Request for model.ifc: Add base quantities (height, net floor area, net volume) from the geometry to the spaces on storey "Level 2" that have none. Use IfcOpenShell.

First a look at what the model holds.

```python
import ifcopenshell
import ifcopenshell.util.element
import ifcopenshell.util.unit

model = ifcopenshell.open("model.ifc")
print(model.schema)
for unit_type in ("LENGTHUNIT", "AREAUNIT", "VOLUMEUNIT"):
    print(unit_type, ifcopenshell.util.unit.calculate_unit_scale(model, unit_type))
storey = next(s for s in model.by_type("IfcBuildingStorey") if s.Name == "Level 2")
spaces = [e for e in ifcopenshell.util.element.get_decomposition(storey) if e.is_a("IfcSpace")]
for e in sorted(spaces, key=lambda e: e.id()):
    print(e.id(), e.is_a(), e.Name, list(ifcopenshell.util.element.get_psets(e, qtos_only=True)), sep=" | ")
```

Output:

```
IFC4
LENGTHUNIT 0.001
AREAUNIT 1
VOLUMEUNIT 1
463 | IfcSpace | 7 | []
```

```python
import ifcopenshell
import ifcopenshell.api.pset
import ifcopenshell.geom
import ifcopenshell.util.element
import ifcopenshell.util.shape
import ifcopenshell.util.unit

model = ifcopenshell.open("model.ifc")
unit_scale = ifcopenshell.util.unit.calculate_unit_scale(model)
area_scale = ifcopenshell.util.unit.calculate_unit_scale(model, "AREAUNIT")
volume_scale = ifcopenshell.util.unit.calculate_unit_scale(model, "VOLUMEUNIT")
settings = ifcopenshell.geom.settings()

storey = next(s for s in model.by_type("IfcBuildingStorey") if s.Name == "Level 2")
spaces = [e for e in ifcopenshell.util.element.get_decomposition(storey) if e.is_a("IfcSpace")]

for e in sorted(spaces, key=lambda e: e.id()):
    if ifcopenshell.util.element.get_psets(e, qtos_only=True, should_inherit=False):
        continue
    # Geometry comes back in metres, in the element's own axes.
    shape = ifcopenshell.geom.create_shape(settings, e)
    values = {
        "Height": ifcopenshell.util.shape.get_z(shape.geometry) / unit_scale,
        "NetFloorArea": ifcopenshell.util.shape.get_footprint_area(shape.geometry) / area_scale,
        "NetVolume": ifcopenshell.util.shape.get_volume(shape.geometry) / volume_scale,
    }
    qto = ifcopenshell.api.pset.add_qto(model, product=e, name="Qto_SpaceBaseQuantities")
    ifcopenshell.api.pset.edit_qto(model, qto=qto, properties=values)
    print(e.id(), {k: round(v, 3) for k, v in values.items()})

model.write("model-out.ifc")
```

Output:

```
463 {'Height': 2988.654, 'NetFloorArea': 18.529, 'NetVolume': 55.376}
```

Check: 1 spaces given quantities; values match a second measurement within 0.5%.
